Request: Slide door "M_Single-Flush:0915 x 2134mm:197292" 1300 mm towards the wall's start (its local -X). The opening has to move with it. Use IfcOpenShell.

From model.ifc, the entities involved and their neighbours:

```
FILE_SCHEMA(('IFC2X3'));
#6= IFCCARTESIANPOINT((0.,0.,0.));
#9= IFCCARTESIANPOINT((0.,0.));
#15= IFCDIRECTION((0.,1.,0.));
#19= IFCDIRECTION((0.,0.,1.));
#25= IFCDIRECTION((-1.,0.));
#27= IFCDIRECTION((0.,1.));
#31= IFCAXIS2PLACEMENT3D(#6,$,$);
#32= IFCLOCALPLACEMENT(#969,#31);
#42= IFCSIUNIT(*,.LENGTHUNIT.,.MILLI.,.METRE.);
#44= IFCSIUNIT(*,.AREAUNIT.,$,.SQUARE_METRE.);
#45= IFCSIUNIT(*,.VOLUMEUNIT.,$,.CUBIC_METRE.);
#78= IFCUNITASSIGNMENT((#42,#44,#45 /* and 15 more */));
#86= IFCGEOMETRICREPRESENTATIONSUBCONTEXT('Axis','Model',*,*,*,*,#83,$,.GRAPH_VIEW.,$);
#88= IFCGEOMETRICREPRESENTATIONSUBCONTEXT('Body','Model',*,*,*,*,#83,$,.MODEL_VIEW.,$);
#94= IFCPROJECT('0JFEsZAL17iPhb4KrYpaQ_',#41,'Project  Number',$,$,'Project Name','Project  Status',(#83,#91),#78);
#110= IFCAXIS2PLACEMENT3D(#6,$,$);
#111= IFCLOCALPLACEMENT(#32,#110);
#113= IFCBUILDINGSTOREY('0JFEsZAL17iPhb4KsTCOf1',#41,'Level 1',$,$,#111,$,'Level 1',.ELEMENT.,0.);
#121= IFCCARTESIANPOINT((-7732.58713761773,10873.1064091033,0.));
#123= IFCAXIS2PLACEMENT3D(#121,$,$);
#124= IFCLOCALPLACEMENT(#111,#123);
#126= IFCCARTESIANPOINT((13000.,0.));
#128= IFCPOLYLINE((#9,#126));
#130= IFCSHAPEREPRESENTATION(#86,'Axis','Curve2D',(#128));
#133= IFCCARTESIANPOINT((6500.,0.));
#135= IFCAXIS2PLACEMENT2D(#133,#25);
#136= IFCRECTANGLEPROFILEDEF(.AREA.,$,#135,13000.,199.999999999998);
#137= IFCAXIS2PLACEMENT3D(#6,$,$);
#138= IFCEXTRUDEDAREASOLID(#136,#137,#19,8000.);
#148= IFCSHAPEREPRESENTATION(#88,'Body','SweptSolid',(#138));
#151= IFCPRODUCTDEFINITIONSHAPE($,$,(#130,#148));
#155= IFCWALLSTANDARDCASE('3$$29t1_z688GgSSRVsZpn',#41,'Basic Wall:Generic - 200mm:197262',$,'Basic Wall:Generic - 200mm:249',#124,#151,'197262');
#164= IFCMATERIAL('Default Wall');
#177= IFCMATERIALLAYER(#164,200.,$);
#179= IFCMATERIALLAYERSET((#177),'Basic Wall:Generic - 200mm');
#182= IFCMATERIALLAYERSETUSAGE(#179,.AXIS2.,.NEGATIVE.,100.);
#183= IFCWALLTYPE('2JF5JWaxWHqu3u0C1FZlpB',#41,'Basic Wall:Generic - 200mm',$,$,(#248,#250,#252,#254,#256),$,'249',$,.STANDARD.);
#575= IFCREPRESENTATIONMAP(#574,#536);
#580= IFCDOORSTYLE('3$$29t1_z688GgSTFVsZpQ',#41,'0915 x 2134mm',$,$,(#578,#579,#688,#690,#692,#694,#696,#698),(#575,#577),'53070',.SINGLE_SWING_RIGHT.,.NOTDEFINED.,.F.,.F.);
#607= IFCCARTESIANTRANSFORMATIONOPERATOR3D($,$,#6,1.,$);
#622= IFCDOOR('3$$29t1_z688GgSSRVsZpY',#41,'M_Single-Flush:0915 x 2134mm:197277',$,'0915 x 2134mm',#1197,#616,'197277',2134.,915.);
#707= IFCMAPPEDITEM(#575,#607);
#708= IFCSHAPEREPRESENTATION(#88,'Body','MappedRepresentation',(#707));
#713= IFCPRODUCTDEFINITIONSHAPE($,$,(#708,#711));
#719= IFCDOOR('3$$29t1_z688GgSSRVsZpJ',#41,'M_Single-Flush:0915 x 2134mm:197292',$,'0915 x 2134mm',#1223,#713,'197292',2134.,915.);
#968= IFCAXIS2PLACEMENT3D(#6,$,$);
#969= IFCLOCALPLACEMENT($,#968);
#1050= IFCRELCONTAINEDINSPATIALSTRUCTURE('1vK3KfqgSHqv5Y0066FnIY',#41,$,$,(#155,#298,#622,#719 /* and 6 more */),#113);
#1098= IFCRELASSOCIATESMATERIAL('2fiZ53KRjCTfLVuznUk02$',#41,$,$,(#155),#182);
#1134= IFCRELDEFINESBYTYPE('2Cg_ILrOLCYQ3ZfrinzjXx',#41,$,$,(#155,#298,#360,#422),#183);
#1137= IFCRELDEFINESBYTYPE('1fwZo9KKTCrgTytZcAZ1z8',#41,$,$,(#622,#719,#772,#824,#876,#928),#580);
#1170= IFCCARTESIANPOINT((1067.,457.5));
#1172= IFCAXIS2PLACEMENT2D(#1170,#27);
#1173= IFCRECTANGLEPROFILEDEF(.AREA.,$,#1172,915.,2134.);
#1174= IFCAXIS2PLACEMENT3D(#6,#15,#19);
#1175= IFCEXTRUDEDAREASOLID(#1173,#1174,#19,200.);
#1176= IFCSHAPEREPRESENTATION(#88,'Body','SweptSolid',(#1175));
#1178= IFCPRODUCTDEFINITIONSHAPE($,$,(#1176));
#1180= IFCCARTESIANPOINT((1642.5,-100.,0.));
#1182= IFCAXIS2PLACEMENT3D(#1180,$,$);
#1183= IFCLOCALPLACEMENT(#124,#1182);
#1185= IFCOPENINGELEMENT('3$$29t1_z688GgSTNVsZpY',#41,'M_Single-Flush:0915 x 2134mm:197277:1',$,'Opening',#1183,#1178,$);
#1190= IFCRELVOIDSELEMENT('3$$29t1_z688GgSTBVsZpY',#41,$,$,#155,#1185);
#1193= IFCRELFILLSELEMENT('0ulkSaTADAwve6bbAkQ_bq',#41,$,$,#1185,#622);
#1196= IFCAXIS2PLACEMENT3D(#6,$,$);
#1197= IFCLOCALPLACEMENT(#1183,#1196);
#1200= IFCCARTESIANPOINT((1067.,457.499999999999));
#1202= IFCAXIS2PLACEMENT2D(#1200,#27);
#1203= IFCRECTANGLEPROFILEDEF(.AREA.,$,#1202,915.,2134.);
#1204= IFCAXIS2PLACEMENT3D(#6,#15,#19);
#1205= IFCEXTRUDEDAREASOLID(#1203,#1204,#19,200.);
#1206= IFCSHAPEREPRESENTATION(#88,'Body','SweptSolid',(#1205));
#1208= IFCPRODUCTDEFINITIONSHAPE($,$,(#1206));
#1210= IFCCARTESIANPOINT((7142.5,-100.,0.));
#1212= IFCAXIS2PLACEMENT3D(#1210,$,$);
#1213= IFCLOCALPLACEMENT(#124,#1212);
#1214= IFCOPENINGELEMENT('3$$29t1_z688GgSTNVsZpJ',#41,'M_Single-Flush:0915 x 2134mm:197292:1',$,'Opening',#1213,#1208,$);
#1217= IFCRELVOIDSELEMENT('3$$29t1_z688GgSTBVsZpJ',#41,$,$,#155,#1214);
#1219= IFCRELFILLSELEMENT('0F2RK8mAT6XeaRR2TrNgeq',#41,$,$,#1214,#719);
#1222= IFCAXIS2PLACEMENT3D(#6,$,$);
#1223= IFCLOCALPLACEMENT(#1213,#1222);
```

```python
import ifcopenshell
import ifcopenshell.api.geometry
import ifcopenshell.util.placement
import ifcopenshell.util.unit

model = ifcopenshell.open("model.ifc")
unit_scale = ifcopenshell.util.unit.calculate_unit_scale(model)

door = model.by_id(719)
opening = door.FillsVoids[0].RelatingOpeningElement
wall = opening.VoidsElements[0].RelatingBuildingElement

wall_matrix = ifcopenshell.util.placement.get_local_placement(wall.ObjectPlacement)
shift = wall_matrix[:3, 0] * -1.3 / unit_scale
before = ifcopenshell.util.placement.get_local_placement(door.ObjectPlacement)[:3, 3].copy()

# The door is placed relative to its opening, so it follows when the opening moves.
matrix = ifcopenshell.util.placement.get_local_placement(opening.ObjectPlacement)
matrix[:3, 3] += shift
ifcopenshell.api.geometry.edit_object_placement(
    model, product=opening, matrix=matrix, is_si=False, should_transform_children=True
)

after = ifcopenshell.util.placement.get_local_placement(door.ObjectPlacement)[:3, 3]
print("door moved by", (after - before).round(3) + 0.0)

model.write("model-out.ifc")
```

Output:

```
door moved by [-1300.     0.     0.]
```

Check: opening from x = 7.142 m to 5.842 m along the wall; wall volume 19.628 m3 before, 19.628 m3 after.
